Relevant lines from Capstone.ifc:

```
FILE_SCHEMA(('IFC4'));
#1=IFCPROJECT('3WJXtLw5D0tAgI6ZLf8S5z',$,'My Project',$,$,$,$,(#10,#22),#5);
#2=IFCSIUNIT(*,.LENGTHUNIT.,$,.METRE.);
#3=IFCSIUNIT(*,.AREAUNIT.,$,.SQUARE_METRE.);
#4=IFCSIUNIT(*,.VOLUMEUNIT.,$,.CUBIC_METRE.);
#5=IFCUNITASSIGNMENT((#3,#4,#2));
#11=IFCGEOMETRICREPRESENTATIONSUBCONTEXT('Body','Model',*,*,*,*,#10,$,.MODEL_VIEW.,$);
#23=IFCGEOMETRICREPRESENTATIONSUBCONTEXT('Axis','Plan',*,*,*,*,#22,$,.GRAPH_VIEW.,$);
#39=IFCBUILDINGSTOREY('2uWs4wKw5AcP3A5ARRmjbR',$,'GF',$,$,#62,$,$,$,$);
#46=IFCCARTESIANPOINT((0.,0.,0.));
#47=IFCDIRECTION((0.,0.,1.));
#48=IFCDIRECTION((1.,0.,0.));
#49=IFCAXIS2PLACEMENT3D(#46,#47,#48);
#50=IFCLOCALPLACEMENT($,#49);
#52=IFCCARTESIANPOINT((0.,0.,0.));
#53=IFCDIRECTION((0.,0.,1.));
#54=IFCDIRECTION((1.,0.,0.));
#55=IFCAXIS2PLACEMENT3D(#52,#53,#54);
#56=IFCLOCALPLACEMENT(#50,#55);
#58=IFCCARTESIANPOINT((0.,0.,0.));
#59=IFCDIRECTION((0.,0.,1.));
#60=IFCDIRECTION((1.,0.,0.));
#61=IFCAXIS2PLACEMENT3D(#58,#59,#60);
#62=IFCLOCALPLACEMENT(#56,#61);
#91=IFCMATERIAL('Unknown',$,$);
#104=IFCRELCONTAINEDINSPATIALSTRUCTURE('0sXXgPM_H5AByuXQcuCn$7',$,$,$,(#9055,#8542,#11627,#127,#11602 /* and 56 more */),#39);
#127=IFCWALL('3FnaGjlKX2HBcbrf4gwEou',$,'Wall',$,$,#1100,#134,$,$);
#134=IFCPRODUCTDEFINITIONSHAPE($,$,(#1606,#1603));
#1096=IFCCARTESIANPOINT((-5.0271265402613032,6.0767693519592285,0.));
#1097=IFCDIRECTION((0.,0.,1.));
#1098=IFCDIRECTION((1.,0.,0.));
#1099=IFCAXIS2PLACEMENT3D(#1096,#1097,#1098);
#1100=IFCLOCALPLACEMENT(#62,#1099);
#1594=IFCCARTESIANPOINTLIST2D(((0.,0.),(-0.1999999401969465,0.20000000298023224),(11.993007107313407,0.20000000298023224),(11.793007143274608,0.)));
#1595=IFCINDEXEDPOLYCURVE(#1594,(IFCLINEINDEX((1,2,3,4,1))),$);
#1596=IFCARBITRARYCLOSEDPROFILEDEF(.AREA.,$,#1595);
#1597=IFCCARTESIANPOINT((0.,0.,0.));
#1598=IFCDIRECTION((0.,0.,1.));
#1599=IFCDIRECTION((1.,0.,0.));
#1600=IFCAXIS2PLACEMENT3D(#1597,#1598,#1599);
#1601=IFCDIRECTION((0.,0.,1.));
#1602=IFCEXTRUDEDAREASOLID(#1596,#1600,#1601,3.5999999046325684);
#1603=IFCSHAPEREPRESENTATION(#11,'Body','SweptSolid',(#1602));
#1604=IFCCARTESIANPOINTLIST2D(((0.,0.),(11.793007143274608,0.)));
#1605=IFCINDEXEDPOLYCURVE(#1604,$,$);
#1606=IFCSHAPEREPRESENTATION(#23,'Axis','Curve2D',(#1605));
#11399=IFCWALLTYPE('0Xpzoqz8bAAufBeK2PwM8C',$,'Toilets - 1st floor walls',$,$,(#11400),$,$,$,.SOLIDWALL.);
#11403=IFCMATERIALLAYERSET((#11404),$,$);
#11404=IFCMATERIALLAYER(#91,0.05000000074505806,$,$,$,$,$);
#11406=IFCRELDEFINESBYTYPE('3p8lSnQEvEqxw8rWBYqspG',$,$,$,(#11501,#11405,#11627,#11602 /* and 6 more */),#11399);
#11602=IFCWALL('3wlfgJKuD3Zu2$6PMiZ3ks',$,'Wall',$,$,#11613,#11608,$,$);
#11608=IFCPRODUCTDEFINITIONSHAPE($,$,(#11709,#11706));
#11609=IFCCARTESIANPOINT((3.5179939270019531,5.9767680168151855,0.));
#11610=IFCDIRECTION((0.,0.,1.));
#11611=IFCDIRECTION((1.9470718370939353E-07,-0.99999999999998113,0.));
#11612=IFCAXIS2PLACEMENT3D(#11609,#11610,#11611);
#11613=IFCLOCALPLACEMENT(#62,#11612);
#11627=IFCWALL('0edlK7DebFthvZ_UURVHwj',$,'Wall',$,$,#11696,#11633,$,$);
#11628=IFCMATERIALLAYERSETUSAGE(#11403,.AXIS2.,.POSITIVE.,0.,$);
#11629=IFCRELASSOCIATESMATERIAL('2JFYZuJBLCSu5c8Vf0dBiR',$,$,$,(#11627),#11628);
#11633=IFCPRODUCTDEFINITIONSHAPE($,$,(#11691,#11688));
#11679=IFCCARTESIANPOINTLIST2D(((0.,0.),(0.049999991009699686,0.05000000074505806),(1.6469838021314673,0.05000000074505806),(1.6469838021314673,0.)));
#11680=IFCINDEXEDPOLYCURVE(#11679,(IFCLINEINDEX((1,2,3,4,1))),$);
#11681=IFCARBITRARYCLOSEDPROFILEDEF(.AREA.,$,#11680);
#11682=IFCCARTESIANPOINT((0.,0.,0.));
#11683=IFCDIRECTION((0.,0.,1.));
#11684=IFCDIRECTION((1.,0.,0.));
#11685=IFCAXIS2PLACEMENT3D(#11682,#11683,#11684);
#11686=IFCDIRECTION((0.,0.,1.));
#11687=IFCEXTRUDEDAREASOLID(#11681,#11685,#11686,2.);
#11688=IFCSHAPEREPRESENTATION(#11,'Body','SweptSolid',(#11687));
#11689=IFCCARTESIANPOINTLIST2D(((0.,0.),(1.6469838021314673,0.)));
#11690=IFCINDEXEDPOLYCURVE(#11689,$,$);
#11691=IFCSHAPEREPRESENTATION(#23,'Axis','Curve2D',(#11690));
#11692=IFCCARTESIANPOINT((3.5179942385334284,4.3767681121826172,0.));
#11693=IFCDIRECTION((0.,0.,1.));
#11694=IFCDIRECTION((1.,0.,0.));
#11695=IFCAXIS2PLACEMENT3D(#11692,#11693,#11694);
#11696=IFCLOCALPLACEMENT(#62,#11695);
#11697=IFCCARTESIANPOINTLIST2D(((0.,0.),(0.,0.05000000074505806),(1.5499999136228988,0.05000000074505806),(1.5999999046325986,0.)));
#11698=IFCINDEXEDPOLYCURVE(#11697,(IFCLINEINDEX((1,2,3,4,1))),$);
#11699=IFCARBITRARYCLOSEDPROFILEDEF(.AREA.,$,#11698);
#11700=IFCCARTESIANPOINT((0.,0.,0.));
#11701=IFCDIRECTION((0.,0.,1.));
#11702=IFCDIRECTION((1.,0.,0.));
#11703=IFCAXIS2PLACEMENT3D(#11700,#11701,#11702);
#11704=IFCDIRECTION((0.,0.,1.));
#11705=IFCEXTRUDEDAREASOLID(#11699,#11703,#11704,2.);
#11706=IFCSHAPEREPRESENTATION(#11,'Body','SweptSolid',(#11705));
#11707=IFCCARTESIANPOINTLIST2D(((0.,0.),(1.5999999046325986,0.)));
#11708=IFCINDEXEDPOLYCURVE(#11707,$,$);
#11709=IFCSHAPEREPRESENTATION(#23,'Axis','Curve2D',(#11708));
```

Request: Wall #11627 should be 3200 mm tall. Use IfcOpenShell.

```python
import ifcopenshell
import ifcopenshell.geom
import ifcopenshell.util.representation
import ifcopenshell.util.shape
import ifcopenshell.util.unit

model = ifcopenshell.open("Capstone.ifc")
unit_scale = ifcopenshell.util.unit.calculate_unit_scale(model)
settings = ifcopenshell.geom.settings()


def volume(element):
    """Net volume in cubic metres, openings subtracted."""
    shape = ifcopenshell.geom.create_shape(settings, element)
    return ifcopenshell.util.shape.get_volume(shape.geometry)


wall = model.by_id(11627)
before = volume(wall)

body = ifcopenshell.util.representation.get_representation(wall, "Model", "Body")
solid = body.Items[0]
old_height = solid.Depth
solid.Depth = 3.2 / unit_scale
after = volume(wall)

print(f"height {old_height:g} -> {solid.Depth:g}, volume {before:.3f} -> {after:.3f} m3")

model.write("Capstone_updated.ifc")
```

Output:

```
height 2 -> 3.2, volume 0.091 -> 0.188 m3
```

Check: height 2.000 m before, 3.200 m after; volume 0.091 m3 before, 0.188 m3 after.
